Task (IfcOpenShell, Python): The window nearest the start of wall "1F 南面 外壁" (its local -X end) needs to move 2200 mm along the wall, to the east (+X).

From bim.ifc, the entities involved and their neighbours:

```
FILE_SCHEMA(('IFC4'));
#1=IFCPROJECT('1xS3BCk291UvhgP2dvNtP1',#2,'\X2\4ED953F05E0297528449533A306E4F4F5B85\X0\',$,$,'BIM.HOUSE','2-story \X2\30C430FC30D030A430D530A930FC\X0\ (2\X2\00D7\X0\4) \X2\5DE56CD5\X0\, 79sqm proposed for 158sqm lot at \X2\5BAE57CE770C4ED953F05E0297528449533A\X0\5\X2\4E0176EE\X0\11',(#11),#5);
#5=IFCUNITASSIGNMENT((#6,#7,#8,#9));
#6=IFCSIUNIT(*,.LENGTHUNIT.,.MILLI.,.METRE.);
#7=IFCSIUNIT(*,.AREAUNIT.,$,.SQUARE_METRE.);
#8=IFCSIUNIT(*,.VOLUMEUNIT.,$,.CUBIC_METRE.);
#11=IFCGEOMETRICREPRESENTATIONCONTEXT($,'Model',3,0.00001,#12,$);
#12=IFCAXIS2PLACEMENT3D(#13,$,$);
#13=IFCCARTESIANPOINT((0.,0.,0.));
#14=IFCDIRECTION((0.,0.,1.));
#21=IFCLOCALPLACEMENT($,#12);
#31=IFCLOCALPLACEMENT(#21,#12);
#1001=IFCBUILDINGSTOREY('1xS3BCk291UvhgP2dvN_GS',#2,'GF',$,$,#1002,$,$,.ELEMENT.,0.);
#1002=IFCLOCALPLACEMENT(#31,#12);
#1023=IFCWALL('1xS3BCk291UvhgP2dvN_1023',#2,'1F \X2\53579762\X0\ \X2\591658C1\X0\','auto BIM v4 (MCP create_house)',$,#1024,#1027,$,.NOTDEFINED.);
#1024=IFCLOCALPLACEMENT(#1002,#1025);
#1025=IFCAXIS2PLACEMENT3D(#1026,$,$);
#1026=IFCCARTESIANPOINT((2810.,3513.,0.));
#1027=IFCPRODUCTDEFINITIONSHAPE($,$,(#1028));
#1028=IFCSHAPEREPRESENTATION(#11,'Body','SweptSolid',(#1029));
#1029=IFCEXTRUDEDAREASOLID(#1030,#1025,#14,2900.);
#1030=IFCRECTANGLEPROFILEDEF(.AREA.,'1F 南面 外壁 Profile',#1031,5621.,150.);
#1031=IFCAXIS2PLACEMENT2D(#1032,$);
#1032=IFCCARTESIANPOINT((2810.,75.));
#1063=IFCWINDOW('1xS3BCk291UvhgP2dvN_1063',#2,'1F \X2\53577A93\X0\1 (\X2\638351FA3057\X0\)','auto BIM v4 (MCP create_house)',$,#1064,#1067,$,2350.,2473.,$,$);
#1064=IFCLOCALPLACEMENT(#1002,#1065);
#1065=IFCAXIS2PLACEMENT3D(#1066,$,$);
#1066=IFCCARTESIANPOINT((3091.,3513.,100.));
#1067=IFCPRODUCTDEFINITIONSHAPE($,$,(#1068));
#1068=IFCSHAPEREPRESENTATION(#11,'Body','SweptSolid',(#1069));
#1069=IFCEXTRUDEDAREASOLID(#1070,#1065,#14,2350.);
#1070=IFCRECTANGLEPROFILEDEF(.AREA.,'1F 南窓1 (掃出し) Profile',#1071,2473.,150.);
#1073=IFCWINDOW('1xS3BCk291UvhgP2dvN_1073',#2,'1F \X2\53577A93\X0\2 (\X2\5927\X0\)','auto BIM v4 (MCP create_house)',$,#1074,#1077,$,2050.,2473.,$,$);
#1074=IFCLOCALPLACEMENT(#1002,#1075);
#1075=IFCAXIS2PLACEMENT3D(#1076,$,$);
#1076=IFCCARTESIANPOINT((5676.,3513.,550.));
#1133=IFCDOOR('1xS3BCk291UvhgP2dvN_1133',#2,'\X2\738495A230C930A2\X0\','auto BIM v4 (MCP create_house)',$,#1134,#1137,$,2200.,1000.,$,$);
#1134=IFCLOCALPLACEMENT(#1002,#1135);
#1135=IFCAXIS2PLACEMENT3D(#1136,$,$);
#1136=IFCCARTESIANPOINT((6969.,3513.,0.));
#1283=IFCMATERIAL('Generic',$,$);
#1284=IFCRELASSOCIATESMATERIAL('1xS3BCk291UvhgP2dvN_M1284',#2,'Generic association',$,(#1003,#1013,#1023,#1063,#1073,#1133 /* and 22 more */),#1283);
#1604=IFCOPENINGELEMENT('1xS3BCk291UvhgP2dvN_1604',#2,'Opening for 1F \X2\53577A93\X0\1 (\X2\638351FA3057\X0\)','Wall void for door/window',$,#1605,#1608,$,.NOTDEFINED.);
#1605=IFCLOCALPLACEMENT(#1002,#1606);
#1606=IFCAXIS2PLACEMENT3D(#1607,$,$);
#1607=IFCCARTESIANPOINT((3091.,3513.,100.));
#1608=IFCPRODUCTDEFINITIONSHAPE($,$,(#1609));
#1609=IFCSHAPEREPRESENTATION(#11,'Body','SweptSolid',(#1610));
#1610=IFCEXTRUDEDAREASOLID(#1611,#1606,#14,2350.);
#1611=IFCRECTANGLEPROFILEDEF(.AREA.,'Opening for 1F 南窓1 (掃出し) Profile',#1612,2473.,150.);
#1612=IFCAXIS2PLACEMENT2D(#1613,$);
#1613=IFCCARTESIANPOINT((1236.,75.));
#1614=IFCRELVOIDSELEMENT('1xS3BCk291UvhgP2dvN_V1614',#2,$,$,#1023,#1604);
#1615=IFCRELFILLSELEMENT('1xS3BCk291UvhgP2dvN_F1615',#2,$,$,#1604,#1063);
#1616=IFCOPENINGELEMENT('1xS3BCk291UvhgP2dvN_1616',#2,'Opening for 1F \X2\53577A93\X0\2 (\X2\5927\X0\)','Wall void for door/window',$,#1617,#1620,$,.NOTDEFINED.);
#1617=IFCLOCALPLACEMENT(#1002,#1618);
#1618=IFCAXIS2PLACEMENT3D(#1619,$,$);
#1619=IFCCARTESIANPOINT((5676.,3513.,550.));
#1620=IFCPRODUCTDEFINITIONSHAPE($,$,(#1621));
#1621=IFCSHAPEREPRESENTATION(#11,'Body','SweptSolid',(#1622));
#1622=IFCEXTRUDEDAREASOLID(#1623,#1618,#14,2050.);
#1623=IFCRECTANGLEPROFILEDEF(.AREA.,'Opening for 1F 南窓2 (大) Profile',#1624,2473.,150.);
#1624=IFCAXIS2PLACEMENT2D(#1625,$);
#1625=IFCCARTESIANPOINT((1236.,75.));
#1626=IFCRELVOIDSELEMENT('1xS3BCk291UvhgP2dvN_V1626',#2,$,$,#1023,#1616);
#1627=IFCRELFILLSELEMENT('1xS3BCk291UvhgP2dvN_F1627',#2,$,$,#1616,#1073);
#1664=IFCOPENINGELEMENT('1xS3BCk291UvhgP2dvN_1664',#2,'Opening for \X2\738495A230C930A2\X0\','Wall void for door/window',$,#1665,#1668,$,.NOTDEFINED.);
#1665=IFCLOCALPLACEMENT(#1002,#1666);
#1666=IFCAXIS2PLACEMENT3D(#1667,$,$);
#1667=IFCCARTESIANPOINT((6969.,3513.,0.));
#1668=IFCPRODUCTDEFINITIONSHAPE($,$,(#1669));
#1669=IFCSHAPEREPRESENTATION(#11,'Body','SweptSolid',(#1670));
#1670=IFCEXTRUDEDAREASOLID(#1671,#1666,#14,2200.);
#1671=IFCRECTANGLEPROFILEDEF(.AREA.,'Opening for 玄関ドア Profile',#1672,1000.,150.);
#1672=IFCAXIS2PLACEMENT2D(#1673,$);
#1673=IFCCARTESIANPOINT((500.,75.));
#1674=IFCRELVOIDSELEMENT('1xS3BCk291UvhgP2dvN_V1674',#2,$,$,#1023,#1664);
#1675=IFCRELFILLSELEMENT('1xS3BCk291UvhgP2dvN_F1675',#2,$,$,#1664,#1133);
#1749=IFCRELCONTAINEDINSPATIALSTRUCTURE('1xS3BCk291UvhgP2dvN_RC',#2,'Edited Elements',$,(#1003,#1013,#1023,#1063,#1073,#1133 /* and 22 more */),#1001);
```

```python
import ifcopenshell
import ifcopenshell.api.geometry
import ifcopenshell.util.placement
import ifcopenshell.util.unit

model = ifcopenshell.open("bim.ifc")
unit_scale = ifcopenshell.util.unit.calculate_unit_scale(model)

window = model.by_guid("1xS3BCk291UvhgP2dvN_1063")
opening = window.FillsVoids[0].RelatingOpeningElement
wall = opening.VoidsElements[0].RelatingBuildingElement

wall_matrix = ifcopenshell.util.placement.get_local_placement(wall.ObjectPlacement)
shift = wall_matrix[:3, 0] * 2.2 / unit_scale
before = ifcopenshell.util.placement.get_local_placement(window.ObjectPlacement)[:3, 3].copy()

# The window is not placed relative to its opening, so move both.
for product in (opening, window):
    matrix = ifcopenshell.util.placement.get_local_placement(product.ObjectPlacement)
    matrix[:3, 3] += shift
    ifcopenshell.api.geometry.edit_object_placement(model, product=product, matrix=matrix, is_si=False)

after = ifcopenshell.util.placement.get_local_placement(window.ObjectPlacement)[:3, 3]
print("window moved by", (after - before).round(3) + 0.0)

model.write("bim_rev.ifc")
```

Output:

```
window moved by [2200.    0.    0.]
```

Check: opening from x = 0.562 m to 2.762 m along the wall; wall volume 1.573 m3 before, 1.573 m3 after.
